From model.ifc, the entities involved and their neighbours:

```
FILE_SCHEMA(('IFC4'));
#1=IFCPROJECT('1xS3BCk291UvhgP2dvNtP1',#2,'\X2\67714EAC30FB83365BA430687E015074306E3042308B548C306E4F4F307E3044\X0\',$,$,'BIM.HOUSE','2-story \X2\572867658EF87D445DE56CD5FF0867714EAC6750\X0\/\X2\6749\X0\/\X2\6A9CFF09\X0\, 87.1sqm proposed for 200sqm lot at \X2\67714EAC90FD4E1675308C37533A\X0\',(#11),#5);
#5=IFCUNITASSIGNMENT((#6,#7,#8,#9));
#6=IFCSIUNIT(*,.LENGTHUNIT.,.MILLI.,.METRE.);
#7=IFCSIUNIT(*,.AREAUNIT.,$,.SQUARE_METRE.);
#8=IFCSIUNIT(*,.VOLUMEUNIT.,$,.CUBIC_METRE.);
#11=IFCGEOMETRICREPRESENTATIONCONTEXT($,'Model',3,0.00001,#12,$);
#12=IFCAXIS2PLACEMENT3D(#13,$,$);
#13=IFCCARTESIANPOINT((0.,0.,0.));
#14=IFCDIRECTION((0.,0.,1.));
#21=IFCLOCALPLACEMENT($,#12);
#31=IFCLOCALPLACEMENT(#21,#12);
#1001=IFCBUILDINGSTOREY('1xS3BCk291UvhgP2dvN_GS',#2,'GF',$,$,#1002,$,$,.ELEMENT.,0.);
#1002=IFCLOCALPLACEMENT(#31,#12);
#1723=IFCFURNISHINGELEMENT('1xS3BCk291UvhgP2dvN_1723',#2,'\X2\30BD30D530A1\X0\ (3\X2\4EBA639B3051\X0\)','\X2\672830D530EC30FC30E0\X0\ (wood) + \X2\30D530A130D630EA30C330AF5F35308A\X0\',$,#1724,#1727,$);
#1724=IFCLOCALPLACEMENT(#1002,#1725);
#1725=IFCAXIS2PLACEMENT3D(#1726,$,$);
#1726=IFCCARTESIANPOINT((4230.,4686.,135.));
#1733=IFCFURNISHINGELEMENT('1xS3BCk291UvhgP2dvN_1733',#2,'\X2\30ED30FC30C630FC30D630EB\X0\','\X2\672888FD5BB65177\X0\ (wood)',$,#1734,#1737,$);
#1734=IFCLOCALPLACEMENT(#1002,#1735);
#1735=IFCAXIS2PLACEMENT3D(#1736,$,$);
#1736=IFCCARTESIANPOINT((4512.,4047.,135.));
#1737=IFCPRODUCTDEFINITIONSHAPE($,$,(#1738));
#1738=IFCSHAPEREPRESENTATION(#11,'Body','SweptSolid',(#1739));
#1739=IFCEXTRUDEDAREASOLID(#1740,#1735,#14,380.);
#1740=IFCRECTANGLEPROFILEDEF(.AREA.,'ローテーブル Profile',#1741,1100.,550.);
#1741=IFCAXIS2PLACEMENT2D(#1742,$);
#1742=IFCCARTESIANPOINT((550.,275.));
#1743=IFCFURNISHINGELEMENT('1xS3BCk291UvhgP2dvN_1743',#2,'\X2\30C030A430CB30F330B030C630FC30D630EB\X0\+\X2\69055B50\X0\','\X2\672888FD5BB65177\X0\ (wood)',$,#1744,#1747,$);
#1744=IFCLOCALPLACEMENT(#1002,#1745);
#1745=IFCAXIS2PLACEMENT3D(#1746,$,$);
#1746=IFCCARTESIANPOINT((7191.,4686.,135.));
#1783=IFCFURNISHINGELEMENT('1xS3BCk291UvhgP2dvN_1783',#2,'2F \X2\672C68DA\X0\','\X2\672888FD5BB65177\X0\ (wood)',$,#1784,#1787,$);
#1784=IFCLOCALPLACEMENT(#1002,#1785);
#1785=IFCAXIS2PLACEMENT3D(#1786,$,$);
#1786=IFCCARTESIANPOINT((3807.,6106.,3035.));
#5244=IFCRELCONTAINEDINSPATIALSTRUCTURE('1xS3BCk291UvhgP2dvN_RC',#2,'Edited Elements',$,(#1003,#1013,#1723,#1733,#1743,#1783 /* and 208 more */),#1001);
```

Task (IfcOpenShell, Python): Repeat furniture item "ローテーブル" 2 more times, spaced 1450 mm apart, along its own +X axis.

```python
import ifcopenshell
import ifcopenshell.api.geometry
import ifcopenshell.api.root
import ifcopenshell.util.element
import ifcopenshell.util.placement
import ifcopenshell.util.unit

model = ifcopenshell.open("model.ifc")
unit_scale = ifcopenshell.util.unit.calculate_unit_scale(model)


def reuse_history(source, copy):
    """copy_class also copies each property set's owner history, people and application; keep the originals."""
    for rel in copy.IsDefinedBy:
        if rel.is_a("IfcRelDefinesByProperties") and (history := rel.RelatingPropertyDefinition.OwnerHistory):
            rel.RelatingPropertyDefinition.OwnerHistory = source.OwnerHistory
            ifcopenshell.util.element.remove_deep2(model, history)


source = model.by_id(1733)
base = ifcopenshell.util.placement.get_local_placement(source.ObjectPlacement)
step = base[:3, 0] * 1.45 / unit_scale

for i in range(1, 3):
    copy = ifcopenshell.api.root.copy_class(model, product=source)
    copy.Representation = ifcopenshell.util.element.copy_deep(
        model, source.Representation, exclude=["IfcGeometricRepresentationContext", "IfcRepresentationMap"]
    )
    reuse_history(source, copy)
    matrix = base.copy()
    matrix[:3, 3] += i * step
    print("added at", matrix[:3, 3].round(3) + 0.0)
    ifcopenshell.api.geometry.edit_object_placement(model, product=copy, matrix=matrix, is_si=False)

model.write("model_updated.ifc")
```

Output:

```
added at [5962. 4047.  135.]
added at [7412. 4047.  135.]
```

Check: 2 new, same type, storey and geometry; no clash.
